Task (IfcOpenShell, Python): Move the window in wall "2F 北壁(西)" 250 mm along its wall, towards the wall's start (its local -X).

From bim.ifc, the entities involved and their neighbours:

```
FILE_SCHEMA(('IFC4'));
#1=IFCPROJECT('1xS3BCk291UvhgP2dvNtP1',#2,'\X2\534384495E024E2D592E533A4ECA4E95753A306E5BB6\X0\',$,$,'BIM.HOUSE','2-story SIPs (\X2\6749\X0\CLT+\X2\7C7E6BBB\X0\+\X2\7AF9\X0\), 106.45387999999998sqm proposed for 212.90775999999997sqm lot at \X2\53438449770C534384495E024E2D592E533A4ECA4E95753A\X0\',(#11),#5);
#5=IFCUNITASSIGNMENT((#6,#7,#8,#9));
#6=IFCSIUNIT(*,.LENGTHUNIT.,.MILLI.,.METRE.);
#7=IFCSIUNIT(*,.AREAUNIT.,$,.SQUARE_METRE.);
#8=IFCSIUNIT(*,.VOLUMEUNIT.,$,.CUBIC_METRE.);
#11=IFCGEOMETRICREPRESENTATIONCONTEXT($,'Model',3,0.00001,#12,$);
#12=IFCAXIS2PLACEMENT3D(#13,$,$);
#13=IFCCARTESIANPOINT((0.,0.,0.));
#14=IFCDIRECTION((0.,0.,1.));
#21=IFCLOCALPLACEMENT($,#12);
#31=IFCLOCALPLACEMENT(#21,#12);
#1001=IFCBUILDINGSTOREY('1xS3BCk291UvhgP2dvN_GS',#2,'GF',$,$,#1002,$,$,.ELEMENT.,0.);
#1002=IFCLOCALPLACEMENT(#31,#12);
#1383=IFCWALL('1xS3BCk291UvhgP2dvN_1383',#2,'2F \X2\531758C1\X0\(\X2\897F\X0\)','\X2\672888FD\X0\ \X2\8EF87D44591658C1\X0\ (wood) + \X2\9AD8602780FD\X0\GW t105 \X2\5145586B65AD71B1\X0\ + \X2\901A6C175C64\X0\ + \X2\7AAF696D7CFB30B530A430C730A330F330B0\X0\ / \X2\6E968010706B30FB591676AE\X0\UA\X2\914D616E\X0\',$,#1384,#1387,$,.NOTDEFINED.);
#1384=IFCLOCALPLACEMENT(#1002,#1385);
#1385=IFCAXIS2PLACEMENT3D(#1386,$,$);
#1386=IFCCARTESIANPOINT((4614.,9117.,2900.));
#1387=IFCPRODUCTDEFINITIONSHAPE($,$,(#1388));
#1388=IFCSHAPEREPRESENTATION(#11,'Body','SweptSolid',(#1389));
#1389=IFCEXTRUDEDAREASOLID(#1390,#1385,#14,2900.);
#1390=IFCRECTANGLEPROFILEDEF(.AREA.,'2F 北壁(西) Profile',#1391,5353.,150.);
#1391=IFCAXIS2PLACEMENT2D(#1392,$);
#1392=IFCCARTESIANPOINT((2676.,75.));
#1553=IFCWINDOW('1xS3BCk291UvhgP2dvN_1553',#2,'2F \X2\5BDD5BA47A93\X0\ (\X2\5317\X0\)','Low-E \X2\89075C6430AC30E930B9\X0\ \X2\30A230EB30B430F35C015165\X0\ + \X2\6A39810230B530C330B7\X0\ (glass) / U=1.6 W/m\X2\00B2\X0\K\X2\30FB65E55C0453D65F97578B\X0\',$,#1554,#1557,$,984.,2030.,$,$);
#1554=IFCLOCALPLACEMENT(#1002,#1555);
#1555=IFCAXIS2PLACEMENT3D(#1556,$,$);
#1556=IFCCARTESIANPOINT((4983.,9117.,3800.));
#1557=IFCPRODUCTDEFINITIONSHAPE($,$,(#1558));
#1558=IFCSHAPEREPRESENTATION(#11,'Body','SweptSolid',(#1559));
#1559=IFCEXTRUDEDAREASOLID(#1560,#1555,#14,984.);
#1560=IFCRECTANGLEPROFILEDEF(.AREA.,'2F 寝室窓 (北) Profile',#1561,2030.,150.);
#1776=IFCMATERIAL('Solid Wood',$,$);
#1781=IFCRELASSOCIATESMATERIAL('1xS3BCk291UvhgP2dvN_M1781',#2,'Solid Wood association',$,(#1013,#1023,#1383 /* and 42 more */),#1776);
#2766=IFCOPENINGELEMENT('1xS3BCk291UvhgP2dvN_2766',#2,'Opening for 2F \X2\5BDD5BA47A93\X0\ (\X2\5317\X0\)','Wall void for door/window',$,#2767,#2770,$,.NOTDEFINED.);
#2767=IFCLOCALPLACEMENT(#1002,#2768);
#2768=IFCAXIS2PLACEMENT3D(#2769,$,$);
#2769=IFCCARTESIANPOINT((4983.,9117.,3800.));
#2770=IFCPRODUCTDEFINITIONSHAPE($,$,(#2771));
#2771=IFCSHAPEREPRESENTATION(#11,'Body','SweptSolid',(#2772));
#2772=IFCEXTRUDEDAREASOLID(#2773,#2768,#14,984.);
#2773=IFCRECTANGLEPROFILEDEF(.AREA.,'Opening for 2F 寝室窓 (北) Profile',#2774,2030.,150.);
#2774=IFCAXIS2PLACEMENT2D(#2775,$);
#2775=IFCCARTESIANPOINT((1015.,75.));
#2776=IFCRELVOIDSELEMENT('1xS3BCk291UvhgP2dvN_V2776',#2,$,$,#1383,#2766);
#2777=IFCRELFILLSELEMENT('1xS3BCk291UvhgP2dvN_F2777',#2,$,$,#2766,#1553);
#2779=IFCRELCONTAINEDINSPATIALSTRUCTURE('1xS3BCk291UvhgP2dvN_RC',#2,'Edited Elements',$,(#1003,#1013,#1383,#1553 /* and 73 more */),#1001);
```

```python
import ifcopenshell
import ifcopenshell.api.geometry
import ifcopenshell.util.placement
import ifcopenshell.util.unit

model = ifcopenshell.open("bim.ifc")
unit_scale = ifcopenshell.util.unit.calculate_unit_scale(model)

window = model.by_guid("1xS3BCk291UvhgP2dvN_1553")
opening = window.FillsVoids[0].RelatingOpeningElement
wall = opening.VoidsElements[0].RelatingBuildingElement

wall_matrix = ifcopenshell.util.placement.get_local_placement(wall.ObjectPlacement)
shift = wall_matrix[:3, 0] * -0.25 / unit_scale
before = ifcopenshell.util.placement.get_local_placement(window.ObjectPlacement)[:3, 3].copy()

# The window is not placed relative to its opening, so move both.
for product in (opening, window):
    matrix = ifcopenshell.util.placement.get_local_placement(product.ObjectPlacement)
    matrix[:3, 3] += shift
    ifcopenshell.api.geometry.edit_object_placement(model, product=product, matrix=matrix, is_si=False)

after = ifcopenshell.util.placement.get_local_placement(window.ObjectPlacement)[:3, 3]
print("window moved by", (after - before).round(3) + 0.0)

model.write("bim-out.ifc")
```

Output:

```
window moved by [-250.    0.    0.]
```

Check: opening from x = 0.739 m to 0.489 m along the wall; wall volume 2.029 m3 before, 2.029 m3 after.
